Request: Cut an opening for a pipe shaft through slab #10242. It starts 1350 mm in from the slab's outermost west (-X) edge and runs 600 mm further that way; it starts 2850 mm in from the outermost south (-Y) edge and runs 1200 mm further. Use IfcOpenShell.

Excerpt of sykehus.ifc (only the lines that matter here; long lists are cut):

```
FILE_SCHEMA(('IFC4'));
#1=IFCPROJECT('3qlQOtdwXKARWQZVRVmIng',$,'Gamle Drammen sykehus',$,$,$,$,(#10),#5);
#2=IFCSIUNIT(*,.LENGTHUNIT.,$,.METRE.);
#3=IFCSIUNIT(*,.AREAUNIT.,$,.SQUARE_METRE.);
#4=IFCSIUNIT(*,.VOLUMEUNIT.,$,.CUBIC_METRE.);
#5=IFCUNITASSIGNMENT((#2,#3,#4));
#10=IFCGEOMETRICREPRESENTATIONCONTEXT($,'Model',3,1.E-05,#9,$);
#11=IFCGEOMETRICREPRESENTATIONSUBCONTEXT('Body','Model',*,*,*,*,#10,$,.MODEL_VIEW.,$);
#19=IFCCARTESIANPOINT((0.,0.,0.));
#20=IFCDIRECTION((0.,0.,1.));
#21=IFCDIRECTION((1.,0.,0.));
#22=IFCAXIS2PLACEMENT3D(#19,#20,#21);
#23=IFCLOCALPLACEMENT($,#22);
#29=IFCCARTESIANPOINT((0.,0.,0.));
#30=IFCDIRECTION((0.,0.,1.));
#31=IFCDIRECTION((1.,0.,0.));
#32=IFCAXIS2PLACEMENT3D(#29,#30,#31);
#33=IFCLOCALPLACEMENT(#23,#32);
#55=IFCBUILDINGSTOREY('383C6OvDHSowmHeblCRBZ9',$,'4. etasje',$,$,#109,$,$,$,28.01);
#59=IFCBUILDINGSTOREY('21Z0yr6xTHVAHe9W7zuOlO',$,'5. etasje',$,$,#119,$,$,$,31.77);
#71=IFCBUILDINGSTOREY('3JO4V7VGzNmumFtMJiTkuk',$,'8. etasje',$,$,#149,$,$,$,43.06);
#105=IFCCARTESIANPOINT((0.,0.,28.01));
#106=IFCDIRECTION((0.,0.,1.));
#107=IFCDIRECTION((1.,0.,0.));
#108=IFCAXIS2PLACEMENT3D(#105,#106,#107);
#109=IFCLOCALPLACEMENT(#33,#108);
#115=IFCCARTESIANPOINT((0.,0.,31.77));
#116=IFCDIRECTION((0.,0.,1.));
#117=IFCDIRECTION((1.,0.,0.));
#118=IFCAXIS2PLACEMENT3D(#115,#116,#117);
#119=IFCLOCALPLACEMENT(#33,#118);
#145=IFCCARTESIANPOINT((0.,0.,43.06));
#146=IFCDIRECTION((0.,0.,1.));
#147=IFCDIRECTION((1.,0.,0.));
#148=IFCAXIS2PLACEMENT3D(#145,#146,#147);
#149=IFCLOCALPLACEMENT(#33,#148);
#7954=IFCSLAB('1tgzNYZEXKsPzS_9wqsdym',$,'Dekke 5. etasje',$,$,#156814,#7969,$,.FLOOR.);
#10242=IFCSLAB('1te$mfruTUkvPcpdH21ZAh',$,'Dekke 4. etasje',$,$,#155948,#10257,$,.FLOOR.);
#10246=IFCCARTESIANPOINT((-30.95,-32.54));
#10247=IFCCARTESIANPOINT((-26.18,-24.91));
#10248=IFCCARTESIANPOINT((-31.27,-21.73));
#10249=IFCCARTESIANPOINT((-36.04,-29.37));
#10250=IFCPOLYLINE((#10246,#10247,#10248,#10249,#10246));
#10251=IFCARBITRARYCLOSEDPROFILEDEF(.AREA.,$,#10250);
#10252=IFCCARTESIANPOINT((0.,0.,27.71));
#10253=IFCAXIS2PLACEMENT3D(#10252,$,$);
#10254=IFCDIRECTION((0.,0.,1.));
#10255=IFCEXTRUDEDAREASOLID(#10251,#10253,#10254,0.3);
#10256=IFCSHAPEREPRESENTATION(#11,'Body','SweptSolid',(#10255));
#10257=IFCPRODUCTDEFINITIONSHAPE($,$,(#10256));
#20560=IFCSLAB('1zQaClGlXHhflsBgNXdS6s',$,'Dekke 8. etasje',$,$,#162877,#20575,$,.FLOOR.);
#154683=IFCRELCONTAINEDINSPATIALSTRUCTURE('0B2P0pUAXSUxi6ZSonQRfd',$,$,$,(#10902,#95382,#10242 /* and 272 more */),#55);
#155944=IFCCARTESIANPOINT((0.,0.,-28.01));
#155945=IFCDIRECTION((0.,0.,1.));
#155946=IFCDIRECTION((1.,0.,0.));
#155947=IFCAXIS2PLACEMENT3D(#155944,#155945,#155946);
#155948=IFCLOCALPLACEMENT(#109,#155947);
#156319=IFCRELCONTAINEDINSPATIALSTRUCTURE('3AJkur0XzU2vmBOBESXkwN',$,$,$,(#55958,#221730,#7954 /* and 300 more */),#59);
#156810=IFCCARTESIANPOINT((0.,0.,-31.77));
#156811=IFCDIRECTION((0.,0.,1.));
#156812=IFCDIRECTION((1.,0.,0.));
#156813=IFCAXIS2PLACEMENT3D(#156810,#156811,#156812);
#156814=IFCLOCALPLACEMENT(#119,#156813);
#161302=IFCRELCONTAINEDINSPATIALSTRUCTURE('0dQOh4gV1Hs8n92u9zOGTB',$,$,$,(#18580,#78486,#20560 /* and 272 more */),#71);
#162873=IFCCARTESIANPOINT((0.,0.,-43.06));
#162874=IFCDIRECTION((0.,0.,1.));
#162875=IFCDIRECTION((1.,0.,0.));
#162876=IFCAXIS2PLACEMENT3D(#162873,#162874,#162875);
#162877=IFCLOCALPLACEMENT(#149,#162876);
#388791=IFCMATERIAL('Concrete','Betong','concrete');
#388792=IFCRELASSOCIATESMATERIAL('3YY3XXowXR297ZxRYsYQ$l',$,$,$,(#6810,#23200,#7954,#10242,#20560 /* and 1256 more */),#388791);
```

```python
import numpy as np
import ifcopenshell
import ifcopenshell.api.feature
import ifcopenshell.api.geometry
import ifcopenshell.api.root
import ifcopenshell.geom
import ifcopenshell.util.placement
import ifcopenshell.util.representation
import ifcopenshell.util.shape
import ifcopenshell.util.unit

model = ifcopenshell.open("sykehus.ifc")
unit_scale = ifcopenshell.util.unit.calculate_unit_scale(model)
settings = ifcopenshell.geom.settings()


def volume(element):
    """Net volume in cubic metres, openings subtracted."""
    shape = ifcopenshell.geom.create_shape(settings, element)
    return ifcopenshell.util.shape.get_volume(shape.geometry)


slab = model.by_guid("1te$mfruTUkvPcpdH21ZAh")
before = volume(slab)

# Extent in the slab's own axes, in metres. The edges named are its -X and -Y sides.
slab_shape = ifcopenshell.geom.create_shape(settings, slab)
vertices = ifcopenshell.util.shape.get_vertices(slab_shape.geometry)
x_min, y_min, bottom = vertices.min(axis=0)
top = vertices[:, 2].max()

opening = ifcopenshell.api.root.create_entity(model, ifc_class="IfcOpeningElement", name="Pipe shaft opening", predefined_type="OPENING")
context = ifcopenshell.util.representation.get_context(model, "Model", "Body", "MODEL_VIEW")
width, depth = 0.6, 1.2
outline = [(0.0, 0.0), (width, 0.0), (width, depth), (0.0, depth), (0.0, 0.0)]
# Overshoot both faces by 50 mm so the cut is clean.
shape = ifcopenshell.api.geometry.add_slab_representation(
    model, context=context, depth=top - bottom + 0.1, polyline=outline
)
ifcopenshell.api.geometry.assign_representation(model, product=opening, representation=shape)

matrix = ifcopenshell.util.placement.get_local_placement(slab.ObjectPlacement)
matrix[:, 3] = matrix @ np.append(np.array([x_min + 1.35, y_min + 2.85, bottom - 0.05]) / unit_scale, 1.0)
ifcopenshell.api.geometry.edit_object_placement(model, product=opening, matrix=matrix, is_si=False)
ifcopenshell.api.feature.add_feature(model, feature=opening, element=slab)

after = volume(slab)

print(f"slab volume {before:.3f} -> {after:.3f} m3")

model.write("sykehus_edited.ifc")
```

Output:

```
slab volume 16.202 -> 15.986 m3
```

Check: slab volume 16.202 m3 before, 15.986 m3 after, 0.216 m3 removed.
